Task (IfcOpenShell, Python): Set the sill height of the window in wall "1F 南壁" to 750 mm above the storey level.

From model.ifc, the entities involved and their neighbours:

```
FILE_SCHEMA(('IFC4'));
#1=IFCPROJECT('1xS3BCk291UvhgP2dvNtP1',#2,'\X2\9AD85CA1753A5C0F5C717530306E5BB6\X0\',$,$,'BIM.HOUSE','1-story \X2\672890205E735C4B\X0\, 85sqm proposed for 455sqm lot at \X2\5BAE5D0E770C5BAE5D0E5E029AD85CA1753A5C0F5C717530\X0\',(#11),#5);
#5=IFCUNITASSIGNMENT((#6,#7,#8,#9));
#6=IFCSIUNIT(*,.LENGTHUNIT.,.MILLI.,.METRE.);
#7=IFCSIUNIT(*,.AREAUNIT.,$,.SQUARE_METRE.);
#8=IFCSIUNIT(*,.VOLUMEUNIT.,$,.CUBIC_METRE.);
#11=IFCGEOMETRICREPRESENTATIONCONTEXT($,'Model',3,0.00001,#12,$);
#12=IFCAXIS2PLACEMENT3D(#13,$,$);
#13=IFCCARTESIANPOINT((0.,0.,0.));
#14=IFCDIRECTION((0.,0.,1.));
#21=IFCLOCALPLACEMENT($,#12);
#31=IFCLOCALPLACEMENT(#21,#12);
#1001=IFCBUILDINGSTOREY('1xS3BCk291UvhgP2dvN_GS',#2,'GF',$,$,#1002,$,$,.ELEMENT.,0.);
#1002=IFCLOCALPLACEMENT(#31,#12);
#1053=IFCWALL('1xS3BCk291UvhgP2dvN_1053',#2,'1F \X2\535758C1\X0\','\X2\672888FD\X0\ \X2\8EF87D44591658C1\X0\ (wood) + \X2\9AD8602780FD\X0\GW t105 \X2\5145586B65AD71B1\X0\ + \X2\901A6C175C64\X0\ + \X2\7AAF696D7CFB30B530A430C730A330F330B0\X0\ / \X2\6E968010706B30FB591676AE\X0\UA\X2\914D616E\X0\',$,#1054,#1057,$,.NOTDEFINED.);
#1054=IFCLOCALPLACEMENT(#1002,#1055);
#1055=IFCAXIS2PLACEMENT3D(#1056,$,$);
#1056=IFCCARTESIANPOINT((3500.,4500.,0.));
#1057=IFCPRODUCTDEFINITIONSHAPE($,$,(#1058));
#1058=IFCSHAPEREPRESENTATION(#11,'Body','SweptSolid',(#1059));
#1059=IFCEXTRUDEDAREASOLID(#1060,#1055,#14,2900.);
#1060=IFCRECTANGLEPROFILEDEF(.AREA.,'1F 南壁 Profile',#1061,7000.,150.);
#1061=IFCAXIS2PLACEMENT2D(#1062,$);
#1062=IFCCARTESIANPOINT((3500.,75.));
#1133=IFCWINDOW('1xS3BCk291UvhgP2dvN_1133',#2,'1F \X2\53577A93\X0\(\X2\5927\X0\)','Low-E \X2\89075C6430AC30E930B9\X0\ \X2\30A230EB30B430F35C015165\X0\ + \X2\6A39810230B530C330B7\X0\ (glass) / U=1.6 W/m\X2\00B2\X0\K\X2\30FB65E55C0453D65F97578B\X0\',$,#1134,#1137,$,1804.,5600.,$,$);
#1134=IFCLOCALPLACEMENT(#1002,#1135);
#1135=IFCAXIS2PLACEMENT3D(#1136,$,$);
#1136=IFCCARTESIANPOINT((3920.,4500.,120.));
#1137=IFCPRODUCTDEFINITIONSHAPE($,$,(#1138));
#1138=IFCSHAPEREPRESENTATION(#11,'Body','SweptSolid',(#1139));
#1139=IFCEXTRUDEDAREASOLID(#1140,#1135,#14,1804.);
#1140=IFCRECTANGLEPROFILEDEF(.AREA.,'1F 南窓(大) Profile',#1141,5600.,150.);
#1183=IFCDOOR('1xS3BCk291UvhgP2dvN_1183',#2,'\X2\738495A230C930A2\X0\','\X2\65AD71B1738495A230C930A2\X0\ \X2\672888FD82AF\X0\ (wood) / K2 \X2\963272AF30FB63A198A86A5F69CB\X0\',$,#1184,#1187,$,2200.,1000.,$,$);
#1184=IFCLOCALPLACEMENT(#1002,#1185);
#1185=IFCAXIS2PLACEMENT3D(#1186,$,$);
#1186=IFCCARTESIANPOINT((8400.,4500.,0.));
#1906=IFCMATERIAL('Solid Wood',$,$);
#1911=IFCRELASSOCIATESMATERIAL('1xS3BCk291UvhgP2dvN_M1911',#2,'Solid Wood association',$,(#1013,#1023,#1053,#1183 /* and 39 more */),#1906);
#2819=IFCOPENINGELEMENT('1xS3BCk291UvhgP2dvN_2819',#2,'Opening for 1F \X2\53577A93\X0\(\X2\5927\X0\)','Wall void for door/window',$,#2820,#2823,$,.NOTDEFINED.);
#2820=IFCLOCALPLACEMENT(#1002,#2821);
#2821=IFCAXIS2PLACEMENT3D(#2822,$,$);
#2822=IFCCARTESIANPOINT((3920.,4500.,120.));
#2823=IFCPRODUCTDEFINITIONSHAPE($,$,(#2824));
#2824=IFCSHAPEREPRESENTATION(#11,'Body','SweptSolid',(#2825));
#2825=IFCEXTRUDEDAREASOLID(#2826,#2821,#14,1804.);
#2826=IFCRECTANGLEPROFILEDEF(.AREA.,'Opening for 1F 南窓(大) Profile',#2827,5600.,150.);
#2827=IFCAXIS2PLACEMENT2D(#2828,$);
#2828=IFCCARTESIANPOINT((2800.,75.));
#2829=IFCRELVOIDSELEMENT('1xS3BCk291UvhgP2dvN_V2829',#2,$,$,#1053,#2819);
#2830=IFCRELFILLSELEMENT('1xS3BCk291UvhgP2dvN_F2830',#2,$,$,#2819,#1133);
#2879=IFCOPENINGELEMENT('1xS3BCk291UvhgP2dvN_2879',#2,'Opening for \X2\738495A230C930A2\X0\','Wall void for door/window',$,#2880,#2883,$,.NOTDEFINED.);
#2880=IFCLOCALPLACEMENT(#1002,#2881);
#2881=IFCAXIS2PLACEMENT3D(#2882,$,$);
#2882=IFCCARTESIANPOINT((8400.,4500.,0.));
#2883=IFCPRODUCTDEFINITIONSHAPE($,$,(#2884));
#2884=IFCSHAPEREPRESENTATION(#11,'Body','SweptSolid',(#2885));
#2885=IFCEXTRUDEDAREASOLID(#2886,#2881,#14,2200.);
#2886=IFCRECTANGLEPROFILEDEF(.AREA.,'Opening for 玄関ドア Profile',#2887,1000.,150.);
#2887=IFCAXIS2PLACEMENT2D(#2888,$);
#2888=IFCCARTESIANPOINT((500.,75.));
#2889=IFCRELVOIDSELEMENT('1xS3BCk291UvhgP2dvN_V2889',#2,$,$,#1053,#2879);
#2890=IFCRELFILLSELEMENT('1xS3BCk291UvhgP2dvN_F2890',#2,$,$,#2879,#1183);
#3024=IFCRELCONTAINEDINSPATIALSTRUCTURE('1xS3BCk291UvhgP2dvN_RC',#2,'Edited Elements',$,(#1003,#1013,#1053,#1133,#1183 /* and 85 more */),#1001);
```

```python
import numpy as np
import ifcopenshell
import ifcopenshell.api.geometry
import ifcopenshell.geom
import ifcopenshell.util.element
import ifcopenshell.util.placement
import ifcopenshell.util.shape
import ifcopenshell.util.unit

model = ifcopenshell.open("model.ifc")
unit_scale = ifcopenshell.util.unit.calculate_unit_scale(model)

window = model.by_guid("1xS3BCk291UvhgP2dvN_1133")
opening = window.FillsVoids[0].RelatingOpeningElement
storey = ifcopenshell.util.element.get_container(window, ifc_class="IfcBuildingStorey")
level = ifcopenshell.util.placement.get_local_placement(storey.ObjectPlacement)[2, 3]

# The opening's origin need not be at the sill, so measure its lowest point.
shape = ifcopenshell.geom.create_shape(ifcopenshell.geom.settings(), opening)
bottom = ifcopenshell.util.shape.get_shape_bottom_elevation(shape, shape.geometry) / unit_scale
dz = level + 0.75 / unit_scale - bottom

shift = np.array([0.0, 0.0, dz])
# The window is not placed relative to its opening, so move both.
for product in (opening, window):
    matrix = ifcopenshell.util.placement.get_local_placement(product.ObjectPlacement)
    matrix[:3, 3] += shift
    ifcopenshell.api.geometry.edit_object_placement(model, product=product, matrix=matrix, is_si=False)

print(f"moved by {dz * unit_scale:+.3f} m")

model.write("model-out.ifc")
```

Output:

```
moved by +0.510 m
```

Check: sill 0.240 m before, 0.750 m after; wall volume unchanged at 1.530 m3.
